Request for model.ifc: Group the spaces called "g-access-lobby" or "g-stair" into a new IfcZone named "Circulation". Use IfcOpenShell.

First a look at what the model holds.

```python
import ifcopenshell

model = ifcopenshell.open("model.ifc")
print(model.schema)
seen = {}
for space in model.by_type("IfcSpace"):
    seen[space.LongName] = seen.get(space.LongName, 0) + 1
for name, count in sorted(seen.items(), key=str):
    print(count, "x", name)
print("zones:", [z.Name for z in model.by_type("IfcZone")][:20])
```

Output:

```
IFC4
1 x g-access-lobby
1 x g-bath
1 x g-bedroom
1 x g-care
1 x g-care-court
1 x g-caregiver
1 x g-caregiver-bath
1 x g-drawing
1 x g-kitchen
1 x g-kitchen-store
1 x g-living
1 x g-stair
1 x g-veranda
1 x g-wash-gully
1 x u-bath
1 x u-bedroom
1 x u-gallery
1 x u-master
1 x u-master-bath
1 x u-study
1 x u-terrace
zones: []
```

```python
import ifcopenshell
import ifcopenshell.api.group
import ifcopenshell.api.root

model = ifcopenshell.open("model.ifc")

names = {"g-access-lobby", "g-stair"}
spaces = [s for s in model.by_type("IfcSpace") if s.LongName in names]

zone = ifcopenshell.api.root.create_entity(model, ifc_class="IfcZone", name="Circulation")
ifcopenshell.api.group.assign_group(model, products=spaces, group=zone)
print(len(spaces), "spaces in", zone.Name)

model.write("model_updated.ifc")
```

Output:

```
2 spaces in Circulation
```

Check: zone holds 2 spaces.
